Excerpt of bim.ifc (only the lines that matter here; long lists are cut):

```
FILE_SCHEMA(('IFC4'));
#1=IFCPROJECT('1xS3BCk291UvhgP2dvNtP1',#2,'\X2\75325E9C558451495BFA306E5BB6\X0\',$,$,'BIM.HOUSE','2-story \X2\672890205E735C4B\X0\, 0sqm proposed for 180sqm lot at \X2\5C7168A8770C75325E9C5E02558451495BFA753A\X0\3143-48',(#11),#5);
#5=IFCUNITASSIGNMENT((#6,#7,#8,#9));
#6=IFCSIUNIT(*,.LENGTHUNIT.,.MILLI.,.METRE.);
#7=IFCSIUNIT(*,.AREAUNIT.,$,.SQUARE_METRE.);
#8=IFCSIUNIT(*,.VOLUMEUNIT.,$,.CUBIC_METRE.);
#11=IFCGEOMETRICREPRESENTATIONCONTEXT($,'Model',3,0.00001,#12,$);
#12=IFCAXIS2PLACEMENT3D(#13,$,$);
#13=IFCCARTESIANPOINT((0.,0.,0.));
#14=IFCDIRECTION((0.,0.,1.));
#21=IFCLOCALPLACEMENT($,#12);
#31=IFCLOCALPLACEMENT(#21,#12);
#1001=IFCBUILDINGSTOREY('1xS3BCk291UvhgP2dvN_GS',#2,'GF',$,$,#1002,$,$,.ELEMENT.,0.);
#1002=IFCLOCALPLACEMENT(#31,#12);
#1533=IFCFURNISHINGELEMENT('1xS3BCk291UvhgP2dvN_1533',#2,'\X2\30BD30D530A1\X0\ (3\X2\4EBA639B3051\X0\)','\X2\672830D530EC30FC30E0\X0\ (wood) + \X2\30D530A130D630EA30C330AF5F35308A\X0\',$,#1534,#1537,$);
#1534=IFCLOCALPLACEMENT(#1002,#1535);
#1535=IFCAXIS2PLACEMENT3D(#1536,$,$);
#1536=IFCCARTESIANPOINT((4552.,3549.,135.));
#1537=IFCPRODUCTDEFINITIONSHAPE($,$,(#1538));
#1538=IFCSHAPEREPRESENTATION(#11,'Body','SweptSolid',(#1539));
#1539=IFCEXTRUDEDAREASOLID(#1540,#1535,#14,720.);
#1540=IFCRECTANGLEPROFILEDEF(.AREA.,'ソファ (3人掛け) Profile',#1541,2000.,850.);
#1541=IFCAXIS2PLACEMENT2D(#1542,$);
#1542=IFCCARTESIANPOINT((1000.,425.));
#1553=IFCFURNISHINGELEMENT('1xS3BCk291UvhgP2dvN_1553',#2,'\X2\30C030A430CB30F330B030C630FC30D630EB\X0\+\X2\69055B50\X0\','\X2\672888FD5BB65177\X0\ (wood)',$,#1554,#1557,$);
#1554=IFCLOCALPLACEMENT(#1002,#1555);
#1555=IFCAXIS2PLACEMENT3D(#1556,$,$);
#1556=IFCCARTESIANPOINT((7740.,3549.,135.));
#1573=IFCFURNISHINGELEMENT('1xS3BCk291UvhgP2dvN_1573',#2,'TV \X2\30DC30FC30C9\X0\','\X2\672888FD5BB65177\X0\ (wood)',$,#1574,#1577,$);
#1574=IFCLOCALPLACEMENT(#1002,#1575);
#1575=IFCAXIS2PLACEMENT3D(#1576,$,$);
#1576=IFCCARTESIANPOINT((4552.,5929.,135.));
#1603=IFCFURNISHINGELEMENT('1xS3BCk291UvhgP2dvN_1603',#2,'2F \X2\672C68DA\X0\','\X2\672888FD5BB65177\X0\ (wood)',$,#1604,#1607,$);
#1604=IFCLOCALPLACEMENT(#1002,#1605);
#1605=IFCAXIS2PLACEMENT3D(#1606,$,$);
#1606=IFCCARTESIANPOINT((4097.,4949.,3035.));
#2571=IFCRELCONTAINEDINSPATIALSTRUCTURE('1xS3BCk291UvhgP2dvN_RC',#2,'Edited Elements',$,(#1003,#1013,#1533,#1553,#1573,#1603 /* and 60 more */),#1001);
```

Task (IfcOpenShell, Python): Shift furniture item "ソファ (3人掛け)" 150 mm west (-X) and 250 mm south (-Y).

```python
import ifcopenshell
import ifcopenshell.api.geometry
import ifcopenshell.util.placement

model = ifcopenshell.open("bim.ifc")

item = model.by_id(1533)
matrix = ifcopenshell.util.placement.get_local_placement(item.ObjectPlacement)
matrix[0, 3] -= 150.0
matrix[1, 3] -= 250.0
ifcopenshell.api.geometry.edit_object_placement(model, product=item, matrix=matrix, is_si=False)

print(ifcopenshell.util.placement.get_local_placement(item.ObjectPlacement).round(3) + 0.0)

model.write("bim_updated.ifc")
```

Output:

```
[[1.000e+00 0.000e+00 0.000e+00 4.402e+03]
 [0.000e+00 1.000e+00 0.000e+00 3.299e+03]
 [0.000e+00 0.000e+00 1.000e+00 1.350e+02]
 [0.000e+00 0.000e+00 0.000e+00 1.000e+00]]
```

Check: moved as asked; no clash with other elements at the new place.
